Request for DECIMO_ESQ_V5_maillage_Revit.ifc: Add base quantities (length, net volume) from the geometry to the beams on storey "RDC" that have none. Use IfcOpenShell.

First a look at what the model holds.

```python
import ifcopenshell
import ifcopenshell.util.element
import ifcopenshell.util.unit

model = ifcopenshell.open("DECIMO_ESQ_V5_maillage_Revit.ifc")
print(model.schema)
for unit_type in ("LENGTHUNIT", "AREAUNIT", "VOLUMEUNIT"):
    print(unit_type, ifcopenshell.util.unit.calculate_unit_scale(model, unit_type))
storey = next(s for s in model.by_type("IfcBuildingStorey") if s.Name == "RDC")
beams = [e for e in ifcopenshell.util.element.get_decomposition(storey) if e.is_a("IfcBeam")]
for e in sorted(beams, key=lambda e: e.id()):
    print(e.id(), e.is_a(), e.Name, list(ifcopenshell.util.element.get_psets(e, qtos_only=True)), sep=" | ")
```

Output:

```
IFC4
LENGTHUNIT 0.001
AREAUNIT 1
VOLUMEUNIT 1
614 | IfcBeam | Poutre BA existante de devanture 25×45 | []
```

```python
import ifcopenshell
import ifcopenshell.api.pset
import ifcopenshell.geom
import ifcopenshell.util.element
import ifcopenshell.util.shape
import ifcopenshell.util.unit

model = ifcopenshell.open("DECIMO_ESQ_V5_maillage_Revit.ifc")
unit_scale = ifcopenshell.util.unit.calculate_unit_scale(model)
volume_scale = ifcopenshell.util.unit.calculate_unit_scale(model, "VOLUMEUNIT")
settings = ifcopenshell.geom.settings()

storey = next(s for s in model.by_type("IfcBuildingStorey") if s.Name == "RDC")
beams = [e for e in ifcopenshell.util.element.get_decomposition(storey) if e.is_a("IfcBeam")]

for e in sorted(beams, key=lambda e: e.id()):
    if ifcopenshell.util.element.get_psets(e, qtos_only=True, should_inherit=False):
        continue
    # Geometry comes back in metres, in the element's own axes.
    shape = ifcopenshell.geom.create_shape(settings, e)
    values = {
        "Length": ifcopenshell.util.shape.get_max_xyz(shape.geometry) / unit_scale,
        "NetVolume": ifcopenshell.util.shape.get_volume(shape.geometry) / volume_scale,
    }
    qto = ifcopenshell.api.pset.add_qto(model, product=e, name="Qto_BeamBaseQuantities")
    ifcopenshell.api.pset.edit_qto(model, qto=qto, properties=values)
    print(e.id(), {k: round(v, 3) for k, v in values.items()})

model.write("DECIMO_ESQ_V5_maillage_Revit_v2.ifc")
```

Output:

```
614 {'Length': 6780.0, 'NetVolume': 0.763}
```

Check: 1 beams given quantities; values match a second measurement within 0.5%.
